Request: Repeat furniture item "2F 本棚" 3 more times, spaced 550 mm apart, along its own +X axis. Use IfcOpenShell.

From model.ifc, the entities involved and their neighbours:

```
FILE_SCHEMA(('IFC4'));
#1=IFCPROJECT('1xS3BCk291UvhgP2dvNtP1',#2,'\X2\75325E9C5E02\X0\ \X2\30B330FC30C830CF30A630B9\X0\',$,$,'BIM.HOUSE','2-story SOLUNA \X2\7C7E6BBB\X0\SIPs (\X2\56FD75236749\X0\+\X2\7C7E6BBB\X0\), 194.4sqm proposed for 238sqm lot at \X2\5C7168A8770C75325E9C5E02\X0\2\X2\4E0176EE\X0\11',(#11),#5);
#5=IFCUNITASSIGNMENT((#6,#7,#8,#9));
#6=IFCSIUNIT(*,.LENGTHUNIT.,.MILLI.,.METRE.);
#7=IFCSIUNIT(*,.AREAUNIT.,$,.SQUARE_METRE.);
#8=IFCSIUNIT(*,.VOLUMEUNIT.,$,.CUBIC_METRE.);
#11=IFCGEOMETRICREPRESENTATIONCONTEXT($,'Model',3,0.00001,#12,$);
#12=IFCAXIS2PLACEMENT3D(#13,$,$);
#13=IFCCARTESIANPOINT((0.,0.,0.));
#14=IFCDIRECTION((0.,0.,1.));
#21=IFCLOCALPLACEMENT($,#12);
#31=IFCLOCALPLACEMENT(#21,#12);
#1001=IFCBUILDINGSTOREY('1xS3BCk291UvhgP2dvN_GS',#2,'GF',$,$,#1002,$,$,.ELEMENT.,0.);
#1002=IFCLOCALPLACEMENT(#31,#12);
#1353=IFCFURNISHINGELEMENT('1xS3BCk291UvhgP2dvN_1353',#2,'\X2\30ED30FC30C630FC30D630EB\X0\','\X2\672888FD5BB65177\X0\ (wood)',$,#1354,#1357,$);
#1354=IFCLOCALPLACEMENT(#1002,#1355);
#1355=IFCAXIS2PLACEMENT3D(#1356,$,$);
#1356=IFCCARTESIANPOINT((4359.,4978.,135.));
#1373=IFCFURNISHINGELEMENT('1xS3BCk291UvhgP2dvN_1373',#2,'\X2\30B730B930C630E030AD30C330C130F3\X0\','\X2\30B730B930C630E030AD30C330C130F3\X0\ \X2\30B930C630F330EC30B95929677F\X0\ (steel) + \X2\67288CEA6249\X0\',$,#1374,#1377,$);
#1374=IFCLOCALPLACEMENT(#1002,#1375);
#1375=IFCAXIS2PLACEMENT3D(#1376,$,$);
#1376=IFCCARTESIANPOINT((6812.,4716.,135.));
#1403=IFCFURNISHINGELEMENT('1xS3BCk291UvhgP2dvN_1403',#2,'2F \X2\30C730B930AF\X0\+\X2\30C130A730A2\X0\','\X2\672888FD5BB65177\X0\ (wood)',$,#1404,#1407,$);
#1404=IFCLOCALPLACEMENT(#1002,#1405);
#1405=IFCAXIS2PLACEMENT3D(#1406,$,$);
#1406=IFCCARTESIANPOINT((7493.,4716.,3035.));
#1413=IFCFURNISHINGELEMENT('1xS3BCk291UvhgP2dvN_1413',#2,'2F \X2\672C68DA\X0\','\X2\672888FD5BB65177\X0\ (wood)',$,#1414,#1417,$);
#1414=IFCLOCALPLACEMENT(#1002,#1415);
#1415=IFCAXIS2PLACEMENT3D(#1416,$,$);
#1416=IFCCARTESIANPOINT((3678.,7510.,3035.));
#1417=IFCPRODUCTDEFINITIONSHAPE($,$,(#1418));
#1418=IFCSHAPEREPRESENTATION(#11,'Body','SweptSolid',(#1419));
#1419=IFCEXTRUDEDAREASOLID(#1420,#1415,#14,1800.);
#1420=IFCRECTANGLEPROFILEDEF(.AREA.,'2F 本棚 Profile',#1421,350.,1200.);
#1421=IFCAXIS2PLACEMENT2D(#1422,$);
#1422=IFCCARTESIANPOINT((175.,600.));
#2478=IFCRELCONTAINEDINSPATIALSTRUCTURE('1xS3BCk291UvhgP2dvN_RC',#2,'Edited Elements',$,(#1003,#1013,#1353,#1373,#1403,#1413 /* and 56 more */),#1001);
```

```python
import ifcopenshell
import ifcopenshell.api.geometry
import ifcopenshell.api.root
import ifcopenshell.util.element
import ifcopenshell.util.placement

model = ifcopenshell.open("model.ifc")


def reuse_history(source, copy):
    """copy_class also copies each property set's owner history, people and application; keep the originals."""
    for rel in copy.IsDefinedBy:
        if rel.is_a("IfcRelDefinesByProperties") and (history := rel.RelatingPropertyDefinition.OwnerHistory):
            rel.RelatingPropertyDefinition.OwnerHistory = source.OwnerHistory
            ifcopenshell.util.element.remove_deep2(model, history)


source = model.by_guid("1xS3BCk291UvhgP2dvN_1413")
base = ifcopenshell.util.placement.get_local_placement(source.ObjectPlacement)
step = base[:3, 0] * 550.0

for i in range(1, 4):
    copy = ifcopenshell.api.root.copy_class(model, product=source)
    copy.Representation = ifcopenshell.util.element.copy_deep(
        model, source.Representation, exclude=["IfcGeometricRepresentationContext", "IfcRepresentationMap"]
    )
    reuse_history(source, copy)
    matrix = base.copy()
    matrix[:3, 3] += i * step
    print("added at", matrix[:3, 3].round(3) + 0.0)
    ifcopenshell.api.geometry.edit_object_placement(model, product=copy, matrix=matrix, is_si=False)

model.write("model-out.ifc")
```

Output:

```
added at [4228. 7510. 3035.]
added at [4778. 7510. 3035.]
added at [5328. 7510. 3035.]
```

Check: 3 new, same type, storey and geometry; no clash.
